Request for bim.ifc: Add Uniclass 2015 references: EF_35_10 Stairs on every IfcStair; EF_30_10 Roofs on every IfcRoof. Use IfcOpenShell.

First a look at what the model holds.

```python
import ifcopenshell

model = ifcopenshell.open("bim.ifc")
print(model.schema)
print("classifications:", [c.Name for c in model.by_type("IfcClassification")])
for ifc_class in ("IfcDoor", "IfcRoof", "IfcStair", "IfcWall", "IfcWindow"):
    print(ifc_class, len(model.by_type(ifc_class)))
```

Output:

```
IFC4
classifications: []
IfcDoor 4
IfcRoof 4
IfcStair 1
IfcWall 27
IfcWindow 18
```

```python
import ifcopenshell
import ifcopenshell.api.classification

model = ifcopenshell.open("bim.ifc")

system = ifcopenshell.api.classification.add_classification(model, classification="Uniclass 2015")

codes = {
    "IfcStair": ("EF_35_10", "Stairs"),
    "IfcRoof": ("EF_30_10", "Roofs"),
}
for ifc_class, (code, name) in codes.items():
    products = model.by_type(ifc_class)
    ifcopenshell.api.classification.add_reference(
        model, products=products, classification=system, identification=code, name=name
    )
    print(code, len(products))

model.write("bim_edited.ifc")
```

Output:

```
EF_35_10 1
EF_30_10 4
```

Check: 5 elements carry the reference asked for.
